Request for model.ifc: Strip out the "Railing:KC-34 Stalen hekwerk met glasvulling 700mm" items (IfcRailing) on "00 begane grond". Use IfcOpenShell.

First a look at what the model holds.

```python
import ifcopenshell
import ifcopenshell.util.element

model = ifcopenshell.open("model.ifc")
print(model.schema)
storey = next(s for s in model.by_type("IfcBuildingStorey") if s.Name == "00 begane grond")
railings = [e for e in ifcopenshell.util.element.get_decomposition(storey) if e.is_a("IfcRailing")]
seen = {}
for e in railings:
    element_type = ifcopenshell.util.element.get_type(e)
    name = element_type.Name if element_type not in (None, e) else None
    seen[name] = seen.get(name, 0) + 1
for name, count in sorted(seen.items(), key=str):
    print(count, "x", name)
```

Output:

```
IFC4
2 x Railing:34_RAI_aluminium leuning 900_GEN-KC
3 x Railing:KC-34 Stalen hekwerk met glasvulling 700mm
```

```python
import ifcopenshell
import ifcopenshell.api.root
import ifcopenshell.util.element

model = ifcopenshell.open("model.ifc")

storey = next(s for s in model.by_type("IfcBuildingStorey") if s.Name == "00 begane grond")
railings = [e for e in ifcopenshell.util.element.get_decomposition(storey) if e.is_a("IfcRailing")]
targets = [e for e in railings if (t := ifcopenshell.util.element.get_type(e)) not in (None, e) and t.Name == "Railing:KC-34 Stalen hekwerk met glasvulling 700mm"]

for e in targets:
    ifcopenshell.api.root.remove_product(model, product=e)
print(len(targets), "removed")

model.write("model_edited.ifc")
```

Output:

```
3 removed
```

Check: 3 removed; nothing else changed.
